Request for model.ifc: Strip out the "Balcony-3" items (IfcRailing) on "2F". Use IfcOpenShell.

First a look at what the model holds.

```python
import ifcopenshell
import ifcopenshell.util.element

model = ifcopenshell.open("model.ifc")
print(model.schema)
storey = next(s for s in model.by_type("IfcBuildingStorey") if s.Name == "2F")
railings = [e for e in ifcopenshell.util.element.get_decomposition(storey) if e.is_a("IfcRailing")]
seen = {}
for e in railings:
    element_type = ifcopenshell.util.element.get_type(e)
    name = element_type.Name if element_type not in (None, e) else None
    seen[name] = seen.get(name, 0) + 1
for name, count in sorted(seen.items(), key=str):
    print(count, "x", name)
```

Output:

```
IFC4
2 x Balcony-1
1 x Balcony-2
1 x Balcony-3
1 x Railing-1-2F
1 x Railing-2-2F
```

```python
import ifcopenshell
import ifcopenshell.api.root
import ifcopenshell.util.element

model = ifcopenshell.open("model.ifc")

storey = next(s for s in model.by_type("IfcBuildingStorey") if s.Name == "2F")
railings = [e for e in ifcopenshell.util.element.get_decomposition(storey) if e.is_a("IfcRailing")]
targets = [e for e in railings if (t := ifcopenshell.util.element.get_type(e)) not in (None, e) and t.Name == "Balcony-3"]

for e in targets:
    ifcopenshell.api.root.remove_product(model, product=e)
print(len(targets), "removed")

model.write("model_rev.ifc")
```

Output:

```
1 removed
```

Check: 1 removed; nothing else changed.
